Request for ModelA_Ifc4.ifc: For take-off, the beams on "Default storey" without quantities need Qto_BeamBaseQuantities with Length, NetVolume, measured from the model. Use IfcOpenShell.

First a look at what the model holds.

```python
import ifcopenshell
import ifcopenshell.util.element
import ifcopenshell.util.unit

model = ifcopenshell.open("ModelA_Ifc4.ifc")
print(model.schema)
for unit_type in ("LENGTHUNIT", "AREAUNIT", "VOLUMEUNIT"):
    print(unit_type, ifcopenshell.util.unit.calculate_unit_scale(model, unit_type))
storey = next(s for s in model.by_type("IfcBuildingStorey") if s.Name == "Default storey")
beams = [e for e in ifcopenshell.util.element.get_decomposition(storey) if e.is_a("IfcBeam")]
for e in sorted(beams, key=lambda e: e.id()):
    print(e.id(), e.is_a(), e.Name, list(ifcopenshell.util.element.get_psets(e, qtos_only=True)), sep=" | ")
```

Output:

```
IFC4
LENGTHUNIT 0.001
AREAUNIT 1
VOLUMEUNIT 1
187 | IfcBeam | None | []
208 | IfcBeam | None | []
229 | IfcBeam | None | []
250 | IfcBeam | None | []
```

```python
import ifcopenshell
import ifcopenshell.api.pset
import ifcopenshell.geom
import ifcopenshell.util.element
import ifcopenshell.util.shape
import ifcopenshell.util.unit

model = ifcopenshell.open("ModelA_Ifc4.ifc")
unit_scale = ifcopenshell.util.unit.calculate_unit_scale(model)
volume_scale = ifcopenshell.util.unit.calculate_unit_scale(model, "VOLUMEUNIT")
settings = ifcopenshell.geom.settings()

storey = next(s for s in model.by_type("IfcBuildingStorey") if s.Name == "Default storey")
beams = [e for e in ifcopenshell.util.element.get_decomposition(storey) if e.is_a("IfcBeam")]

for e in sorted(beams, key=lambda e: e.id()):
    if ifcopenshell.util.element.get_psets(e, qtos_only=True, should_inherit=False):
        continue
    # Geometry comes back in metres, in the element's own axes.
    shape = ifcopenshell.geom.create_shape(settings, e)
    values = {
        "Length": ifcopenshell.util.shape.get_max_xyz(shape.geometry) / unit_scale,
        "NetVolume": ifcopenshell.util.shape.get_volume(shape.geometry) / volume_scale,
    }
    qto = ifcopenshell.api.pset.add_qto(model, product=e, name="Qto_BeamBaseQuantities")
    ifcopenshell.api.pset.edit_qto(model, qto=qto, properties=values)
    print(e.id(), {k: round(v, 3) for k, v in values.items()})

model.write("ModelA_Ifc4_edited.ifc")
```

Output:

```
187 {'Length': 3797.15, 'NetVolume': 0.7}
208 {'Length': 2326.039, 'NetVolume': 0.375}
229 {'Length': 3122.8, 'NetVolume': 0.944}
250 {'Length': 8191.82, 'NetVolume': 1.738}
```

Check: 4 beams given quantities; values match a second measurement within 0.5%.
